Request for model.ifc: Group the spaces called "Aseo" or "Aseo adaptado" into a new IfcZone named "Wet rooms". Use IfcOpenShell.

First a look at what the model holds.

```python
import ifcopenshell

model = ifcopenshell.open("model.ifc")
print(model.schema)
seen = {}
for space in model.by_type("IfcSpace"):
    seen[space.LongName] = seen.get(space.LongName, 0) + 1
for name, count in sorted(seen.items(), key=str):
    print(count, "x", name)
print("zones:", [z.Name for z in model.by_type("IfcZone")][:20])
```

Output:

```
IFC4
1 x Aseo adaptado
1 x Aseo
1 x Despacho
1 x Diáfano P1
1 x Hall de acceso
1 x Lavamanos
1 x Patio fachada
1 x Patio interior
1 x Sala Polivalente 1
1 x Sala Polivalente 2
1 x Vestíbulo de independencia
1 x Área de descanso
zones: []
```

```python
import ifcopenshell
import ifcopenshell.api.group
import ifcopenshell.api.root

model = ifcopenshell.open("model.ifc")

names = {"Aseo", "Aseo adaptado"}
spaces = [s for s in model.by_type("IfcSpace") if s.LongName in names]

zone = ifcopenshell.api.root.create_entity(model, ifc_class="IfcZone", name="Wet rooms")
ifcopenshell.api.group.assign_group(model, products=spaces, group=zone)
print(len(spaces), "spaces in", zone.Name)

model.write("model_edited.ifc")
```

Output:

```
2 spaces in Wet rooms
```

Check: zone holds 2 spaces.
